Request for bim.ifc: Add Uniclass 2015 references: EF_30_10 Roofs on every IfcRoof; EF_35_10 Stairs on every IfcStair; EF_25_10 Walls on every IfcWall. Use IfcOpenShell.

First a look at what the model holds.

```python
import ifcopenshell

model = ifcopenshell.open("bim.ifc")
print(model.schema)
print("classifications:", [c.Name for c in model.by_type("IfcClassification")])
for ifc_class in ("IfcDoor", "IfcRoof", "IfcStair", "IfcWall", "IfcWindow"):
    print(ifc_class, len(model.by_type(ifc_class)))
```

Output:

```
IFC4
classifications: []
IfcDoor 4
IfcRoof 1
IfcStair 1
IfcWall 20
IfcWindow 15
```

```python
import ifcopenshell
import ifcopenshell.api.classification

model = ifcopenshell.open("bim.ifc")

system = ifcopenshell.api.classification.add_classification(model, classification="Uniclass 2015")

codes = {
    "IfcRoof": ("EF_30_10", "Roofs"),
    "IfcStair": ("EF_35_10", "Stairs"),
    "IfcWall": ("EF_25_10", "Walls"),
}
for ifc_class, (code, name) in codes.items():
    products = model.by_type(ifc_class)
    ifcopenshell.api.classification.add_reference(
        model, products=products, classification=system, identification=code, name=name
    )
    print(code, len(products))

model.write("bim_edited.ifc")
```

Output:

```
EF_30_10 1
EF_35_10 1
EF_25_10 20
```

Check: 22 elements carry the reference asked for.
